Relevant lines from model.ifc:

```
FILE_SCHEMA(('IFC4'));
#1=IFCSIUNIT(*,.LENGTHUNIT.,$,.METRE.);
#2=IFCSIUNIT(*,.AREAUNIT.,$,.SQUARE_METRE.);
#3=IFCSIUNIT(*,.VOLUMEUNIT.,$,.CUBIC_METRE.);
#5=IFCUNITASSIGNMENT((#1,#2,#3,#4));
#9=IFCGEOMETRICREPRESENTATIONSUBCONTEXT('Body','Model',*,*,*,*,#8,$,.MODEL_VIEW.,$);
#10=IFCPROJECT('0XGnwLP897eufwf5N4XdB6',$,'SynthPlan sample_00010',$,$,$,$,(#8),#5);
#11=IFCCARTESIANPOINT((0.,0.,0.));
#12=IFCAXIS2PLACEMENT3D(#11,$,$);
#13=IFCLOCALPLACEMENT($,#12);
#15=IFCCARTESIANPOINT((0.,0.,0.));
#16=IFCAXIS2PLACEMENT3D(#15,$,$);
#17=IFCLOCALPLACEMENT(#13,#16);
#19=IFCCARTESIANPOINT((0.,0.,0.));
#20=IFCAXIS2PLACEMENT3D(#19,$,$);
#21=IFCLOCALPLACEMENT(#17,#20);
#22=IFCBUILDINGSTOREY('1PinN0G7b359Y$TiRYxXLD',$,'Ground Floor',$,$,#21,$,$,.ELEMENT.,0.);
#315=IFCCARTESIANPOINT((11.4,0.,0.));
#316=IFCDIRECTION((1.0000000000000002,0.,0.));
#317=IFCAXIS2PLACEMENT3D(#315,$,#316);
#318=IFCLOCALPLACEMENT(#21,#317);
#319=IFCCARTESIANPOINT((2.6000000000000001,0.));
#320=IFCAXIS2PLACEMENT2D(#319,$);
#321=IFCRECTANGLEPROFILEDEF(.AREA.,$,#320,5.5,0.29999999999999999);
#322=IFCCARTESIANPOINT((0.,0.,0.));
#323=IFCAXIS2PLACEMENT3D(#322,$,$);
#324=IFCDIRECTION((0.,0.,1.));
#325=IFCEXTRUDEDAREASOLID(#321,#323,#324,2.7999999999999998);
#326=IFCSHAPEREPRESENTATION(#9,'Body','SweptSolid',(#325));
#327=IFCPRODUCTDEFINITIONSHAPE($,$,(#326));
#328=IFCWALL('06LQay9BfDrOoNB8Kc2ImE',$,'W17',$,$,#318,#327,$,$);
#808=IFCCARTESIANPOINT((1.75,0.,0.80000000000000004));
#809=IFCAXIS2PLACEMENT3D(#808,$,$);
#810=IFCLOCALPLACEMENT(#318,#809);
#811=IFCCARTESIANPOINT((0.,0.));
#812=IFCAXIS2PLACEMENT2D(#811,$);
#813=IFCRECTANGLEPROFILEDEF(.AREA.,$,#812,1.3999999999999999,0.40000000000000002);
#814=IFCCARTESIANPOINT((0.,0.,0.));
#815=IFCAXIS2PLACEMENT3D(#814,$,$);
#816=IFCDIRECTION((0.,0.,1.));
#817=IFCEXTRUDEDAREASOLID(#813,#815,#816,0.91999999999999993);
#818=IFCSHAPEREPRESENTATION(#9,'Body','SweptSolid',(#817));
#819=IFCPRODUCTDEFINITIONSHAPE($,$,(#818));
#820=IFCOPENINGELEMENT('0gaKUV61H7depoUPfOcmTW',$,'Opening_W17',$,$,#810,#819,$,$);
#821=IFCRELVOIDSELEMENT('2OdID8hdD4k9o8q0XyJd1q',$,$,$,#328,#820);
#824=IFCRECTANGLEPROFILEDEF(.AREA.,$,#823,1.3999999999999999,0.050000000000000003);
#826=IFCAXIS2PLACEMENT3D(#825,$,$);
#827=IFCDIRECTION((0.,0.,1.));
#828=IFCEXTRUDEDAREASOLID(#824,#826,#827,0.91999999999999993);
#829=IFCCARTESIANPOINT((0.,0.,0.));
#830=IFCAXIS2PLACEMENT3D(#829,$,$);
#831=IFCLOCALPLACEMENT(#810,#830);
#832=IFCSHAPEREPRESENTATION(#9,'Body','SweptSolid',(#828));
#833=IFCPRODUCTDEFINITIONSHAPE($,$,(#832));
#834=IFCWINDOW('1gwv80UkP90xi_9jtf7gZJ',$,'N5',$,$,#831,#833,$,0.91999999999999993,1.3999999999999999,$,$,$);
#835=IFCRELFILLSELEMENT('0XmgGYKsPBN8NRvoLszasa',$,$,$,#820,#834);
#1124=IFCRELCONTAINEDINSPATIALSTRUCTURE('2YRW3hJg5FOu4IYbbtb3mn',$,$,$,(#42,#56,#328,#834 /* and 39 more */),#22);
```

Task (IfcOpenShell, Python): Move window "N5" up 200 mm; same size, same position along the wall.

```python
import numpy as np
import ifcopenshell
import ifcopenshell.api.geometry
import ifcopenshell.util.placement
import ifcopenshell.util.unit

model = ifcopenshell.open("model.ifc")
unit_scale = ifcopenshell.util.unit.calculate_unit_scale(model)

window = model.by_id(834)
opening = window.FillsVoids[0].RelatingOpeningElement
dz = 0.2 / unit_scale

shift = np.array([0.0, 0.0, dz])
# The window is placed relative to its opening, so it follows when the opening moves.
matrix = ifcopenshell.util.placement.get_local_placement(opening.ObjectPlacement)
matrix[:3, 3] += shift
ifcopenshell.api.geometry.edit_object_placement(
    model, product=opening, matrix=matrix, is_si=False, should_transform_children=True
)

print(f"moved by {dz * unit_scale:+.3f} m")

model.write("model_v2.ifc")
```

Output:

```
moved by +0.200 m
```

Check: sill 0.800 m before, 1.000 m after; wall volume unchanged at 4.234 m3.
